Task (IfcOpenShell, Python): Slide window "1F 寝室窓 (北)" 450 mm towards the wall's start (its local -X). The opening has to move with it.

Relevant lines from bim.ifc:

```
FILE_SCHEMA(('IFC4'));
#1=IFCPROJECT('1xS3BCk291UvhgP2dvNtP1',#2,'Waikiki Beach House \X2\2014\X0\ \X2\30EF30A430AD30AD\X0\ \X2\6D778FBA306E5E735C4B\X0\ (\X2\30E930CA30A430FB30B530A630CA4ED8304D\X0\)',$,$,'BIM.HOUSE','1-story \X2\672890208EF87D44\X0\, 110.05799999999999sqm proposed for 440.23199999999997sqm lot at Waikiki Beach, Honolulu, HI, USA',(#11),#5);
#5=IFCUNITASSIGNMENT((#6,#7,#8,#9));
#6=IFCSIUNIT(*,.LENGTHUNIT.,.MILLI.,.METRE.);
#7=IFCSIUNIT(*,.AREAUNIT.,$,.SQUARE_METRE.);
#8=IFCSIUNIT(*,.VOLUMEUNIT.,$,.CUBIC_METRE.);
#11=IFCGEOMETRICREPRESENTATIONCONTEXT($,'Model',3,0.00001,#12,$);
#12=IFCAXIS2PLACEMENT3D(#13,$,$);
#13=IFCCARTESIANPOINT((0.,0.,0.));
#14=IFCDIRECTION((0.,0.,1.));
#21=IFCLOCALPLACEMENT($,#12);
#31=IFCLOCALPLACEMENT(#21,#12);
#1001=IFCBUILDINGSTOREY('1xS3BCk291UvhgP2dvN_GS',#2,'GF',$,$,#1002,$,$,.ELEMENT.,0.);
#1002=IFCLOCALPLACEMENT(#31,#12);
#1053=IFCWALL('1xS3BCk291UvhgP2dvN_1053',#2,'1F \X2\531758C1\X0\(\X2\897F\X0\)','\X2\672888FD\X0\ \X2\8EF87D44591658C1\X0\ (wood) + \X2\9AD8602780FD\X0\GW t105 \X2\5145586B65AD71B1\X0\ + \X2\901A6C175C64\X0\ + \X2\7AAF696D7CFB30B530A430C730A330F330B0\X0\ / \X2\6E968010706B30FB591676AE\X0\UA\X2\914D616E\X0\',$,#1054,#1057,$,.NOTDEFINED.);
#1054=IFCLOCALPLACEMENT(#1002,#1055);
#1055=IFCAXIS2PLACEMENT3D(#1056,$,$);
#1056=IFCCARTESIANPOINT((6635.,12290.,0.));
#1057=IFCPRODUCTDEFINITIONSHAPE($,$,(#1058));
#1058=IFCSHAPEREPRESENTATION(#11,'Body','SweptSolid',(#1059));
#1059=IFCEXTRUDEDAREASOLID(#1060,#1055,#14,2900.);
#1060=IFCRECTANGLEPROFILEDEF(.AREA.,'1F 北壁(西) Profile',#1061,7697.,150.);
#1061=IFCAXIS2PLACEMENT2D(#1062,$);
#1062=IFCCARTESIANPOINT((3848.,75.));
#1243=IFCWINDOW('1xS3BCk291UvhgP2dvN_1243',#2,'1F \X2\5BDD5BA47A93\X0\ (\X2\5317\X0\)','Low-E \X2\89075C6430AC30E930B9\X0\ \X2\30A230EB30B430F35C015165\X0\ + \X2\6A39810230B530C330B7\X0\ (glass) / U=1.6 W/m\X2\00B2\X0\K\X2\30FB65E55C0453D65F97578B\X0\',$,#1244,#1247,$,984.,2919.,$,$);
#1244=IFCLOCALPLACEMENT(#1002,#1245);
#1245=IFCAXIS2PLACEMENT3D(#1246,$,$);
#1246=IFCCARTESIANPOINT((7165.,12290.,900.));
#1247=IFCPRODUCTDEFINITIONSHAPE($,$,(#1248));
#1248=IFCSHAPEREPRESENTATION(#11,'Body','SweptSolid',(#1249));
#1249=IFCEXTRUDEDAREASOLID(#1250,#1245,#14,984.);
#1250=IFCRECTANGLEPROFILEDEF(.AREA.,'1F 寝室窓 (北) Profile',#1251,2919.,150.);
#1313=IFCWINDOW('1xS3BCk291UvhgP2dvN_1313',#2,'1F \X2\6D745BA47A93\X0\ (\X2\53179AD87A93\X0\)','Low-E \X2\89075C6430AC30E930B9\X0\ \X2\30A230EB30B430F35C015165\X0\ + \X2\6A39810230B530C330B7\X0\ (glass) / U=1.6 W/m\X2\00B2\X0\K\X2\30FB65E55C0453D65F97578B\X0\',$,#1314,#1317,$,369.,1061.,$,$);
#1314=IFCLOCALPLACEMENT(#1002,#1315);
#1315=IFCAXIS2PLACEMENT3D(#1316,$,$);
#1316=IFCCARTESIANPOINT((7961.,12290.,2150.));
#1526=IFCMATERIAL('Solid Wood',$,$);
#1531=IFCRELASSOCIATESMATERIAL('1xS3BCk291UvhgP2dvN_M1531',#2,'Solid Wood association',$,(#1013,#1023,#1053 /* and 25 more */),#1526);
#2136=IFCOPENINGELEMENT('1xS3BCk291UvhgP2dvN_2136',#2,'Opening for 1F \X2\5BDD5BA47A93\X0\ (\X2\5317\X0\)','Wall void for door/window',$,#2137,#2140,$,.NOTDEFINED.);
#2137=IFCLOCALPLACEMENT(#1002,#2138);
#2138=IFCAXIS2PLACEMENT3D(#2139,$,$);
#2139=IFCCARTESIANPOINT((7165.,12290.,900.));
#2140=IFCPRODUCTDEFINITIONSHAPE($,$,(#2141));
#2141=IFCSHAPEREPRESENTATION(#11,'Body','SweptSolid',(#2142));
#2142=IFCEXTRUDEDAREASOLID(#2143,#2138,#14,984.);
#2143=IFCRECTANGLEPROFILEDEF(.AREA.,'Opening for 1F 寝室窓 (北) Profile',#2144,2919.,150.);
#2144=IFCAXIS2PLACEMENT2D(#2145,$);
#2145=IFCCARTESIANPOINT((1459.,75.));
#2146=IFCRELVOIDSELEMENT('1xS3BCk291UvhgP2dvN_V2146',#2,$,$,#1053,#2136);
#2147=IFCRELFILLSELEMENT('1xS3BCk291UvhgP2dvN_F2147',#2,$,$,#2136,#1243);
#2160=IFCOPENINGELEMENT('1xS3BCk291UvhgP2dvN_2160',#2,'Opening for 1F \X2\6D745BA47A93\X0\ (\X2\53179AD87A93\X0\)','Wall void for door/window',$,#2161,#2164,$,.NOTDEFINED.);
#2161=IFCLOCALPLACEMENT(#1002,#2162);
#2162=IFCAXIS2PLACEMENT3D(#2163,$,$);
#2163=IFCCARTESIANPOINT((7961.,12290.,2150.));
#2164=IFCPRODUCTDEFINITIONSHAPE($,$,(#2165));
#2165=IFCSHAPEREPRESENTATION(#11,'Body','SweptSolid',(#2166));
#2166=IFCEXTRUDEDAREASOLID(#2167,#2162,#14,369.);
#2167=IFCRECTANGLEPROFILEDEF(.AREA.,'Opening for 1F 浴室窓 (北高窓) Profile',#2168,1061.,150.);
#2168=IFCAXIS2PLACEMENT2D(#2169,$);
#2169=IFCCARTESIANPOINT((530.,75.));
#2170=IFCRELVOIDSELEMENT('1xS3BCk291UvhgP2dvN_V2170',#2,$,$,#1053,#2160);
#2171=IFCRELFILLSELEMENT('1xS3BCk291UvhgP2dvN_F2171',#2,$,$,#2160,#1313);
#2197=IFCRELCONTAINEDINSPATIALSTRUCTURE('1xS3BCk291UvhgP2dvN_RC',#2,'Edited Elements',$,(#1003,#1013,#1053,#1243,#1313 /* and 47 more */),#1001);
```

```python
import ifcopenshell
import ifcopenshell.api.geometry
import ifcopenshell.util.placement

model = ifcopenshell.open("bim.ifc")

window = model.by_guid("1xS3BCk291UvhgP2dvN_1243")
opening = window.FillsVoids[0].RelatingOpeningElement
wall = opening.VoidsElements[0].RelatingBuildingElement

wall_matrix = ifcopenshell.util.placement.get_local_placement(wall.ObjectPlacement)
shift = wall_matrix[:3, 0] * -450.0
before = ifcopenshell.util.placement.get_local_placement(window.ObjectPlacement)[:3, 3].copy()

# The window is not placed relative to its opening, so move both.
for product in (opening, window):
    matrix = ifcopenshell.util.placement.get_local_placement(product.ObjectPlacement)
    matrix[:3, 3] += shift
    ifcopenshell.api.geometry.edit_object_placement(model, product=product, matrix=matrix, is_si=False)

after = ifcopenshell.util.placement.get_local_placement(window.ObjectPlacement)[:3, 3]
print("window moved by", (after - before).round(3) + 0.0)

model.write("bim_edited.ifc")
```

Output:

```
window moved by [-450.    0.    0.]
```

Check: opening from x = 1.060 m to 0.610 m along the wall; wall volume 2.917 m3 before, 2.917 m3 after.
